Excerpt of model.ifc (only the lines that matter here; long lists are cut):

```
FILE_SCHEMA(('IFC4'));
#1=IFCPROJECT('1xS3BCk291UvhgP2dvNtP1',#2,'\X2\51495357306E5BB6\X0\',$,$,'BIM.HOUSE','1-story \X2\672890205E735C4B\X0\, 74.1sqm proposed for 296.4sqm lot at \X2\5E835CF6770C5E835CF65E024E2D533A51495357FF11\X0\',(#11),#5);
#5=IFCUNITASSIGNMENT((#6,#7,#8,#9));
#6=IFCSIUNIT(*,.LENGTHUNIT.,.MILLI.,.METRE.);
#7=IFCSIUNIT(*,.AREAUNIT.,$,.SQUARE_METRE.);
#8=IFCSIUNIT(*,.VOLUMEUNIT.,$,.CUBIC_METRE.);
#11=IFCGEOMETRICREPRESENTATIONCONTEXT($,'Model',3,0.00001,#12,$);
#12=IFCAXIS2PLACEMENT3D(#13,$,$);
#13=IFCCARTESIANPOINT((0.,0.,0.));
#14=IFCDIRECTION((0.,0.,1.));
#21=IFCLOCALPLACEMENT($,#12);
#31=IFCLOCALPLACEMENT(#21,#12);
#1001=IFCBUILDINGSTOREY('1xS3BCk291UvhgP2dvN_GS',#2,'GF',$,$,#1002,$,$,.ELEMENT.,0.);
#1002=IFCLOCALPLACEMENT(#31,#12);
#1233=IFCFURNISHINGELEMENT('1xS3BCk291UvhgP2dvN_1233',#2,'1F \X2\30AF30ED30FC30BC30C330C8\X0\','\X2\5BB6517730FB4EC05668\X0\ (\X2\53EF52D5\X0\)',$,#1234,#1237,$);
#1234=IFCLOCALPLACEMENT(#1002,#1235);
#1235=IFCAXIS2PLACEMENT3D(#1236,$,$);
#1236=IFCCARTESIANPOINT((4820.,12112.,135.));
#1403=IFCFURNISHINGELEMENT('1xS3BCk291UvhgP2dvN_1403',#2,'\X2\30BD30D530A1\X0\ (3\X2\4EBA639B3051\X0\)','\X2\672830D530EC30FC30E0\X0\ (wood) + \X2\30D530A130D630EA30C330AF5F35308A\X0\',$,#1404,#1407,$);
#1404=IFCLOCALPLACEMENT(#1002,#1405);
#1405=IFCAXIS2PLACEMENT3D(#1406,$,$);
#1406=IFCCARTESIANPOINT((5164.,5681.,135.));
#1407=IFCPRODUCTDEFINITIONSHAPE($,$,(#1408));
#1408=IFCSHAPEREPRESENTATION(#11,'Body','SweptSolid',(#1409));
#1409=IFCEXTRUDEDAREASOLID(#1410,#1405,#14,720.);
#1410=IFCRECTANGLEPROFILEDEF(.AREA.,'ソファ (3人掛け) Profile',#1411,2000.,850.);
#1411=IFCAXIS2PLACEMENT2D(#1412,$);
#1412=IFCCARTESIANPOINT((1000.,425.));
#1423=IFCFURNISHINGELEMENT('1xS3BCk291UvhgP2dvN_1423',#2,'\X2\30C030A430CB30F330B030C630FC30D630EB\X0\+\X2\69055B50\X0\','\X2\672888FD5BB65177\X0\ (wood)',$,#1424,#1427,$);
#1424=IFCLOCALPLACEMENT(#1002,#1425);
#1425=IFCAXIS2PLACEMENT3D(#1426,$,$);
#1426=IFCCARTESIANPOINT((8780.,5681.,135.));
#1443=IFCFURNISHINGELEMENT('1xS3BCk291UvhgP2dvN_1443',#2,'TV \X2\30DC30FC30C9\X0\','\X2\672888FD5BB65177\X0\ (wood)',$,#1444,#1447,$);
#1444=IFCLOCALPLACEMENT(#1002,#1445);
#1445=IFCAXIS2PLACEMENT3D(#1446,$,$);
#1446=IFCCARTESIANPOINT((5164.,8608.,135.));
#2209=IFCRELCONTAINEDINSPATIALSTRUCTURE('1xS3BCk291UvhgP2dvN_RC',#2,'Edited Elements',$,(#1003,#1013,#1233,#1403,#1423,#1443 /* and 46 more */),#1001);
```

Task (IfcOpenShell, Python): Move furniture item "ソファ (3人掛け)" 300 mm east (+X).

```python
import ifcopenshell
import ifcopenshell.api.geometry
import ifcopenshell.util.placement

model = ifcopenshell.open("model.ifc")

item = model.by_guid("1xS3BCk291UvhgP2dvN_1403")
matrix = ifcopenshell.util.placement.get_local_placement(item.ObjectPlacement)
matrix[0, 3] += 300.0
ifcopenshell.api.geometry.edit_object_placement(model, product=item, matrix=matrix, is_si=False)

print(ifcopenshell.util.placement.get_local_placement(item.ObjectPlacement).round(3) + 0.0)

model.write("model_edited.ifc")
```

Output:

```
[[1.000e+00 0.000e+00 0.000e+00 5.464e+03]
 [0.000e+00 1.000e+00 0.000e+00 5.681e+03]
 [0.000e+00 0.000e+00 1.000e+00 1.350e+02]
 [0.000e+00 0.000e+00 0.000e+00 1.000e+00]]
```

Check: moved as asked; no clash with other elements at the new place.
